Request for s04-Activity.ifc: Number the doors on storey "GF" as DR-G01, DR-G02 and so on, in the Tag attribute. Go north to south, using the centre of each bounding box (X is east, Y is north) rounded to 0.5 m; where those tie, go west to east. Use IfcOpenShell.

First a look at what the model holds.

```python
import ifcopenshell
import ifcopenshell.util.element
import ifcopenshell.util.placement

model = ifcopenshell.open("s04-Activity.ifc")
print(model.schema)
storey = next(s for s in model.by_type("IfcBuildingStorey") if s.Name == "GF")
doors = [e for e in ifcopenshell.util.element.get_decomposition(storey) if e.is_a("IfcDoor")]
for e in sorted(doors, key=lambda e: e.id()):
    origin = ifcopenshell.util.placement.get_local_placement(e.ObjectPlacement)[:3, 3]
    print(e.id(), e.Tag, e.Name, origin.round(2) + 0.0, sep=" | ")
```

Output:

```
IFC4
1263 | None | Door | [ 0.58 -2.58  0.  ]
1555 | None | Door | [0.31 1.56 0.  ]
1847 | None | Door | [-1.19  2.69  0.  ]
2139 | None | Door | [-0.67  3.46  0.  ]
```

```python
import ifcopenshell
import ifcopenshell.geom
import ifcopenshell.util.element
import ifcopenshell.util.shape

model = ifcopenshell.open("s04-Activity.ifc")
settings = ifcopenshell.geom.settings()
settings.set("use-world-coords", True)


def centre(element):
    shape = ifcopenshell.geom.create_shape(settings, element)
    return ifcopenshell.util.shape.get_bbox_centroid(shape.geometry)


storey = next(s for s in model.by_type("IfcBuildingStorey") if s.Name == "GF")
doors = [e for e in ifcopenshell.util.element.get_decomposition(storey) if e.is_a("IfcDoor")]

# Insertion points can sit at a corner or the storey origin, so sort by the geometry (in metres).
centres = {e: centre(e) for e in doors}
doors.sort(key=lambda e: (-round(centres[e][1] / 0.5), centres[e][0]))

for i, e in enumerate(doors, start=1):
    number = f"DR-G{i:02d}"
    e.Tag = number
    print(e.id(), number)

model.write("s04-Activity_updated.ifc")
```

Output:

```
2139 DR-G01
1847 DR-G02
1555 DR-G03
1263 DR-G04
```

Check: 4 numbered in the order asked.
